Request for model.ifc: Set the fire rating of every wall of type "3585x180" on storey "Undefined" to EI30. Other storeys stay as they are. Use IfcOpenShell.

First a look at what the model holds.

```python
import ifcopenshell
import ifcopenshell.util.element

model = ifcopenshell.open("model.ifc")
print(model.schema)
storey = next(s for s in model.by_type("IfcBuildingStorey") if s.Name == "Undefined")
walls = [e for e in ifcopenshell.util.element.get_decomposition(storey) if e.is_a("IfcWall")]
seen = {}
for e in walls:
    element_type = ifcopenshell.util.element.get_type(e)
    key = (element_type.Name if element_type != e and element_type else None, ifcopenshell.util.element.get_pset(e, "Pset_WallCommon", "FireRating"))
    seen[key] = seen.get(key, 0) + 1
for (name, value), count in sorted(seen.items(), key=str):
    print(count, "x", name, "|", value)
```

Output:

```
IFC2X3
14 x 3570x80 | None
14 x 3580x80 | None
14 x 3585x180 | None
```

```python
import ifcopenshell
import ifcopenshell.api.pset
import ifcopenshell.util.element

model = ifcopenshell.open("model.ifc")

storey = next(s for s in model.by_type("IfcBuildingStorey") if s.Name == "Undefined")
walls = [e for e in ifcopenshell.util.element.get_decomposition(storey) if e.is_a("IfcWall")]

count = 0
for e in walls:
    element_type = ifcopenshell.util.element.get_type(e)
    if element_type in (None, e) or element_type.Name != "3585x180":
        continue
    found = ifcopenshell.util.element.get_pset(e, "Pset_WallCommon", should_inherit=False)
    if found:
        pset = model.by_id(found["id"])
        if len(ifcopenshell.util.element.get_elements_by_pset(pset)) > 1:
            pset = ifcopenshell.api.pset.unshare_pset(model, products=[e], pset=pset)[0]
    else:
        pset = ifcopenshell.api.pset.add_pset(model, product=e, name="Pset_WallCommon")
    ifcopenshell.api.pset.edit_pset(model, pset=pset, properties={"FireRating": "EI30"})
    count += 1

print(count, "walls updated")

model.write("model_edited.ifc")
```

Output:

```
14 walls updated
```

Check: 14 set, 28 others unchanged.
